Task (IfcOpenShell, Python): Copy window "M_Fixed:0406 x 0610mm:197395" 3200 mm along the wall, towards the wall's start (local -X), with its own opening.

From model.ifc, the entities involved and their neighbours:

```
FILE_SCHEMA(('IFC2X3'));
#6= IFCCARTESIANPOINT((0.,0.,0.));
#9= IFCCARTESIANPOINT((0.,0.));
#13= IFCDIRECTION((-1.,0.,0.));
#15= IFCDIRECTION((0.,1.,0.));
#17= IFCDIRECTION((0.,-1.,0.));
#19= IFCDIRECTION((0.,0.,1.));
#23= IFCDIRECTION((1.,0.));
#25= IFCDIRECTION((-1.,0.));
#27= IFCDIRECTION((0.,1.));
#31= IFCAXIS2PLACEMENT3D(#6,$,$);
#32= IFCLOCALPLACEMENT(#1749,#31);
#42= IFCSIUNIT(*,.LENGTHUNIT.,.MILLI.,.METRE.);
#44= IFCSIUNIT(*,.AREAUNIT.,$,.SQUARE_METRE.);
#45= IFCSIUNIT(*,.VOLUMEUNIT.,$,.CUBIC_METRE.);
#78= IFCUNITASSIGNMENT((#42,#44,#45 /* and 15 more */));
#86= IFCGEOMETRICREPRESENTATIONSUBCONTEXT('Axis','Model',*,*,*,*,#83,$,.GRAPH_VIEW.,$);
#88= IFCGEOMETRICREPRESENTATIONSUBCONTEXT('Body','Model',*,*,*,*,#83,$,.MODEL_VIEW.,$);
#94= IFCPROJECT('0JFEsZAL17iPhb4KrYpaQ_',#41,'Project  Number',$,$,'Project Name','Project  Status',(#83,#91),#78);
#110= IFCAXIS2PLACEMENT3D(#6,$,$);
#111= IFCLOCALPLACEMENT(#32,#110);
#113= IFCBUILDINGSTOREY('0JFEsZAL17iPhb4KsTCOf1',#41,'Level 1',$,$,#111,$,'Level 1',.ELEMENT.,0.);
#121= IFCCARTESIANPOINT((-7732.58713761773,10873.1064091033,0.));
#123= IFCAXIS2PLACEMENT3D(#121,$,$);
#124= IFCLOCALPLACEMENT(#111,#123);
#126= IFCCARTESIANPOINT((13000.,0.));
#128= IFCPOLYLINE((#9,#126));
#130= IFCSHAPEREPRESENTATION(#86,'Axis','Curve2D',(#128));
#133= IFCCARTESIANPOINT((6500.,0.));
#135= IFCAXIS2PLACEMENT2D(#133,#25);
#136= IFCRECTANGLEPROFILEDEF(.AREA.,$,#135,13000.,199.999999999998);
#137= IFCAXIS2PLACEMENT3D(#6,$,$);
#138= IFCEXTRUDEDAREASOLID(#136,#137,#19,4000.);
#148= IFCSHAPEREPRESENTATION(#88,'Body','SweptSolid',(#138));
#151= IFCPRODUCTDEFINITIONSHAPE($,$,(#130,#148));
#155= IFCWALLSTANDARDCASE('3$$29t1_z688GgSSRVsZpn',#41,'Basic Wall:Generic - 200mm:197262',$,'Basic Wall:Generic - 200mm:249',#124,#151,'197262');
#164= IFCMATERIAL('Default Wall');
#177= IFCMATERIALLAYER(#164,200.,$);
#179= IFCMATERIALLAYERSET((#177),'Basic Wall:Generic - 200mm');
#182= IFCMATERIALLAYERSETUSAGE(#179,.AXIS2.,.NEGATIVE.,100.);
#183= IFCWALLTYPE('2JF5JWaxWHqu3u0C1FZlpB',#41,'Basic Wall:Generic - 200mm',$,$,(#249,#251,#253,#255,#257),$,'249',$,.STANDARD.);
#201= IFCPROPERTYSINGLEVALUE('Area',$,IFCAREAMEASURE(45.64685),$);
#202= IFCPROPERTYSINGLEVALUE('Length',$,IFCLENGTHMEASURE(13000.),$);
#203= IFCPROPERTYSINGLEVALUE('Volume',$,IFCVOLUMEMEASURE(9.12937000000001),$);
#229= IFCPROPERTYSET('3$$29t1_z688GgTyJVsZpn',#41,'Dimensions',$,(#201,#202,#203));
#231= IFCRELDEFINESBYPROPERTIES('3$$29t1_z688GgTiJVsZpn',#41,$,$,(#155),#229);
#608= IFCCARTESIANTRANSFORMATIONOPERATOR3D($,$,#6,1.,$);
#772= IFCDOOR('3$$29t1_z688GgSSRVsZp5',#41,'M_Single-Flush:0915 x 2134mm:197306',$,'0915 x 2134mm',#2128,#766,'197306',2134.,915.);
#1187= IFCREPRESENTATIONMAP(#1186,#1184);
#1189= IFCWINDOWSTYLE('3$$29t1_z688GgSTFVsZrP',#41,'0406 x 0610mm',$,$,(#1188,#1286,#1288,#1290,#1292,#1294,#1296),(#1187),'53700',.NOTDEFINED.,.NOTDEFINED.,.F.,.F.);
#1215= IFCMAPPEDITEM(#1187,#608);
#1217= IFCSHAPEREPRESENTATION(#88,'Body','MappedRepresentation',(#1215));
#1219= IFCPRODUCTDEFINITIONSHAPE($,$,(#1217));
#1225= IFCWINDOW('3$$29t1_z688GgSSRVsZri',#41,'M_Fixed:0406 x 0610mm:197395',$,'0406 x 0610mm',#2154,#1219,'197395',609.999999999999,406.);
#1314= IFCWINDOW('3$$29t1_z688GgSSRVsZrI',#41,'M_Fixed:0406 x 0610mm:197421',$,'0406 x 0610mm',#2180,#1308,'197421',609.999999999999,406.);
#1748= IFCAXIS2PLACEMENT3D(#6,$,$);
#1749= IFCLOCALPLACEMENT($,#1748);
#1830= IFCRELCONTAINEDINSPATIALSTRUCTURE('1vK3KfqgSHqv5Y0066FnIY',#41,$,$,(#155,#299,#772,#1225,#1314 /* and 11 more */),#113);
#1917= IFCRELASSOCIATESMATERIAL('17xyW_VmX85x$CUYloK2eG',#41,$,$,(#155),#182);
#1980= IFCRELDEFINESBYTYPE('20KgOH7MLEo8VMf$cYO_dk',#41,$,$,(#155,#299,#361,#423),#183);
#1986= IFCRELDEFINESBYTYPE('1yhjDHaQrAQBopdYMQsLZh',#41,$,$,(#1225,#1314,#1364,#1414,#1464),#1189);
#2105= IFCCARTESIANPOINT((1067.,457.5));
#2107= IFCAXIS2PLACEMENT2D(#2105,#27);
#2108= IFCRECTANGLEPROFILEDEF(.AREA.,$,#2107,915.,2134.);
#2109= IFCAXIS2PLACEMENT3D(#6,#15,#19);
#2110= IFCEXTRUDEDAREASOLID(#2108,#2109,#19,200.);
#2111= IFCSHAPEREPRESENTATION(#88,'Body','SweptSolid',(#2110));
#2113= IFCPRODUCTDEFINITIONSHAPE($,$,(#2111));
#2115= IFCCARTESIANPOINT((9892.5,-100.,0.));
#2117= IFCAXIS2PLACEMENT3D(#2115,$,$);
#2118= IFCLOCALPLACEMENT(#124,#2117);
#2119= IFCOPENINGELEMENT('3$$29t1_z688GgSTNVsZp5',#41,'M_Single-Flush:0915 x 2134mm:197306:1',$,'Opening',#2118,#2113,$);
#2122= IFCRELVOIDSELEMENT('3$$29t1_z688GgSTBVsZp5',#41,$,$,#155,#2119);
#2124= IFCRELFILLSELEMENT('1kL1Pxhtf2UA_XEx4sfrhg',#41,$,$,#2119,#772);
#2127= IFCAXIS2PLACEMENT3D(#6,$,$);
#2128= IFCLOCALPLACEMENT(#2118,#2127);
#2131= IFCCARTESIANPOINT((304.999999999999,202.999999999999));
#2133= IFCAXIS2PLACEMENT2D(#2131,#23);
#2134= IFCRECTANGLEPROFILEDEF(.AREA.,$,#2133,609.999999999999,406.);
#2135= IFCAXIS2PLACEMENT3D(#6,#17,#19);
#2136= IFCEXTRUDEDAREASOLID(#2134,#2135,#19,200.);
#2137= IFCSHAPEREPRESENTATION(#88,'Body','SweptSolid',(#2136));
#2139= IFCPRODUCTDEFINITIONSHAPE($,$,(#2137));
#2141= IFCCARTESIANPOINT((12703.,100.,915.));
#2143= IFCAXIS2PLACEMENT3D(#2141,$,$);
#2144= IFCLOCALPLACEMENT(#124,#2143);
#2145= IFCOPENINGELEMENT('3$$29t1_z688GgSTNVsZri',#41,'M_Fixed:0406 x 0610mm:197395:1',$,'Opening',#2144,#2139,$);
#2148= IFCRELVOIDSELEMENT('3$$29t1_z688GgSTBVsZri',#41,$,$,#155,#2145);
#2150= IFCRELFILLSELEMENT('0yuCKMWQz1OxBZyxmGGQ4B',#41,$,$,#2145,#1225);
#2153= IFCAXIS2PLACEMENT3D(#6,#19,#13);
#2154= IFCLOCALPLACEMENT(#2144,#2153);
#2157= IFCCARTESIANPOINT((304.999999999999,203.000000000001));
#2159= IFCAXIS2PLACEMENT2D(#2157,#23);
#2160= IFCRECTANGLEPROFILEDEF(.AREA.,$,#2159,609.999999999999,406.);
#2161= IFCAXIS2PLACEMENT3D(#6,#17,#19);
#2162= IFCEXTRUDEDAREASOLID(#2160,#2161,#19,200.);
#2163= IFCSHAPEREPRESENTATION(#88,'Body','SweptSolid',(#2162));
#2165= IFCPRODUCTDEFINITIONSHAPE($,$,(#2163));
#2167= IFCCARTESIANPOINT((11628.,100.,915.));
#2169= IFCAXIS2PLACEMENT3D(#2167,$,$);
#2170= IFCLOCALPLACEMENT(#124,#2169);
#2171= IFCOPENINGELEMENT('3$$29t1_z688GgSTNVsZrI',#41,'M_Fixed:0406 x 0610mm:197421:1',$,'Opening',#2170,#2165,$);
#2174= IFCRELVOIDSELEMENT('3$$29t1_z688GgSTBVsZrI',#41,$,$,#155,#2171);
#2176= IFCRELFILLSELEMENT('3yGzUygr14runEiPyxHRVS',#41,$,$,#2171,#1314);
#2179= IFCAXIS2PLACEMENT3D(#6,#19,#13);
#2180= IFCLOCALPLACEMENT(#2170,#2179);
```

```python
import ifcopenshell
import ifcopenshell.api.feature
import ifcopenshell.api.geometry
import ifcopenshell.api.pset
import ifcopenshell.api.root
import ifcopenshell.geom
import ifcopenshell.util.element
import ifcopenshell.util.placement
import ifcopenshell.util.shape
import ifcopenshell.util.unit

model = ifcopenshell.open("model.ifc")
area_scale = ifcopenshell.util.unit.calculate_unit_scale(model, "AREAUNIT")
volume_scale = ifcopenshell.util.unit.calculate_unit_scale(model, "VOLUMEUNIT")
settings = ifcopenshell.geom.settings()


def volume(element):
    """Net volume in cubic metres, openings subtracted."""
    shape = ifcopenshell.geom.create_shape(settings, element)
    return ifcopenshell.util.shape.get_volume(shape.geometry)


def reuse_history(source, copy):
    """copy_class also copies each property set's owner history, people and application; keep the originals."""
    for rel in copy.IsDefinedBy:
        if rel.is_a("IfcRelDefinesByProperties") and (history := rel.RelatingPropertyDefinition.OwnerHistory):
            rel.RelatingPropertyDefinition.OwnerHistory = source.OwnerHistory
            ifcopenshell.util.element.remove_deep2(model, history)


window = model.by_guid("3$$29t1_z688GgSSRVsZri")
opening = window.FillsVoids[0].RelatingOpeningElement
wall = opening.VoidsElements[0].RelatingBuildingElement
before = volume(wall)
shift = ifcopenshell.util.placement.get_local_placement(wall.ObjectPlacement)[:3, 0] * -3200.0

# copy_class copies the void relationship, type, container and properties, but no geometry.
new_opening = ifcopenshell.api.root.copy_class(model, product=opening)
new_opening.Representation = ifcopenshell.util.element.copy_deep(
    model, opening.Representation, exclude=["IfcGeometricRepresentationContext", "IfcRepresentationMap"]
)
new_opening.Name = "M_Fixed:0406 x 0610mm"
new_window = ifcopenshell.api.root.copy_class(model, product=window)
new_window.Representation = ifcopenshell.util.element.copy_deep(
    model, window.Representation, exclude=["IfcGeometricRepresentationContext", "IfcRepresentationMap"]
)
new_window.Name = "M_Fixed:0406 x 0610mm"
new_window.Tag = None
reuse_history(window, new_window)
fills = ifcopenshell.api.feature.add_filling(model, opening=new_opening, element=new_window)
fills.OwnerHistory = new_window.OwnerHistory  # required in IFC2X3

for old, new in ((opening, new_opening), (window, new_window)):
    matrix = ifcopenshell.util.placement.get_local_placement(old.ObjectPlacement)
    matrix[:3, 3] += shift
    ifcopenshell.api.geometry.edit_object_placement(model, product=new, matrix=matrix, is_si=False)

after = volume(wall)
thickness = 0.2  # wall thickness in metres

# Update the wall's stored quantities.
pset = model.by_id(ifcopenshell.util.element.get_pset(wall, "Dimensions", should_inherit=False)["id"])
ifcopenshell.api.pset.edit_pset(model, pset=pset, properties={
    "Area": model.create_entity("IfcAreaMeasure", after / thickness / area_scale),
    "Volume": model.create_entity("IfcVolumeMeasure", after / volume_scale),
})

print(f"wall volume {before:.3f} -> {after:.3f} m3")

model.write("model_updated.ifc")
```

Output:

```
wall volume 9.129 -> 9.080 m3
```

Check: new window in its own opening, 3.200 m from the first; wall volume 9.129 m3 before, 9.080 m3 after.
